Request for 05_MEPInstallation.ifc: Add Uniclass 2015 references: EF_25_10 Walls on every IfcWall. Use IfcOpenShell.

First a look at what the model holds.

```python
import ifcopenshell

model = ifcopenshell.open("05_MEPInstallation.ifc")
print(model.schema)
print("classifications:", [c.Name for c in model.by_type("IfcClassification")])
for ifc_class in ("IfcDoor", "IfcRoof", "IfcStair", "IfcWall", "IfcWindow"):
    print(ifc_class, len(model.by_type(ifc_class)))
```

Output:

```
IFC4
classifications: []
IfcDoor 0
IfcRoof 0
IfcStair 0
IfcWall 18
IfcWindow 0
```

```python
import ifcopenshell
import ifcopenshell.api.classification

model = ifcopenshell.open("05_MEPInstallation.ifc")

system = ifcopenshell.api.classification.add_classification(model, classification="Uniclass 2015")

codes = {
    "IfcWall": ("EF_25_10", "Walls"),
}
for ifc_class, (code, name) in codes.items():
    products = model.by_type(ifc_class)
    ifcopenshell.api.classification.add_reference(
        model, products=products, classification=system, identification=code, name=name
    )
    print(code, len(products))

model.write("05_MEPInstallation-out.ifc")
```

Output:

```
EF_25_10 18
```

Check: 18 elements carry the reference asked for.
